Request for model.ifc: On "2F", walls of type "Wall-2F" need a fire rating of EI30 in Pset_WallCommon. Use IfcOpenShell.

First a look at what the model holds.

```python
import ifcopenshell
import ifcopenshell.util.element

model = ifcopenshell.open("model.ifc")
print(model.schema)
storey = next(s for s in model.by_type("IfcBuildingStorey") if s.Name == "2F")
walls = [e for e in ifcopenshell.util.element.get_decomposition(storey) if e.is_a("IfcWall")]
seen = {}
for e in walls:
    element_type = ifcopenshell.util.element.get_type(e)
    key = (element_type.Name if element_type != e and element_type else None, ifcopenshell.util.element.get_pset(e, "Pset_WallCommon", "FireRating"))
    seen[key] = seen.get(key, 0) + 1
for (name, value), count in sorted(seen.items(), key=str):
    print(count, "x", name, "|", value)
```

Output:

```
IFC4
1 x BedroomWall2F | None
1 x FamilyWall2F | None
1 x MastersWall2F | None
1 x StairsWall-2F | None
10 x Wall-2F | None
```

```python
import ifcopenshell
import ifcopenshell.api.pset
import ifcopenshell.util.element

model = ifcopenshell.open("model.ifc")

storey = next(s for s in model.by_type("IfcBuildingStorey") if s.Name == "2F")
walls = [e for e in ifcopenshell.util.element.get_decomposition(storey) if e.is_a("IfcWall")]

count = 0
for e in walls:
    element_type = ifcopenshell.util.element.get_type(e)
    if element_type in (None, e) or element_type.Name != "Wall-2F":
        continue
    # add_pset returns the element's existing set when there is one.
    pset = ifcopenshell.api.pset.add_pset(model, product=e, name="Pset_WallCommon")
    ifcopenshell.api.pset.edit_pset(model, pset=pset, properties={"FireRating": "EI30"})
    count += 1

print(count, "walls updated")

model.write("model-out.ifc")
```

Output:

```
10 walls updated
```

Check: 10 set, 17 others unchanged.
